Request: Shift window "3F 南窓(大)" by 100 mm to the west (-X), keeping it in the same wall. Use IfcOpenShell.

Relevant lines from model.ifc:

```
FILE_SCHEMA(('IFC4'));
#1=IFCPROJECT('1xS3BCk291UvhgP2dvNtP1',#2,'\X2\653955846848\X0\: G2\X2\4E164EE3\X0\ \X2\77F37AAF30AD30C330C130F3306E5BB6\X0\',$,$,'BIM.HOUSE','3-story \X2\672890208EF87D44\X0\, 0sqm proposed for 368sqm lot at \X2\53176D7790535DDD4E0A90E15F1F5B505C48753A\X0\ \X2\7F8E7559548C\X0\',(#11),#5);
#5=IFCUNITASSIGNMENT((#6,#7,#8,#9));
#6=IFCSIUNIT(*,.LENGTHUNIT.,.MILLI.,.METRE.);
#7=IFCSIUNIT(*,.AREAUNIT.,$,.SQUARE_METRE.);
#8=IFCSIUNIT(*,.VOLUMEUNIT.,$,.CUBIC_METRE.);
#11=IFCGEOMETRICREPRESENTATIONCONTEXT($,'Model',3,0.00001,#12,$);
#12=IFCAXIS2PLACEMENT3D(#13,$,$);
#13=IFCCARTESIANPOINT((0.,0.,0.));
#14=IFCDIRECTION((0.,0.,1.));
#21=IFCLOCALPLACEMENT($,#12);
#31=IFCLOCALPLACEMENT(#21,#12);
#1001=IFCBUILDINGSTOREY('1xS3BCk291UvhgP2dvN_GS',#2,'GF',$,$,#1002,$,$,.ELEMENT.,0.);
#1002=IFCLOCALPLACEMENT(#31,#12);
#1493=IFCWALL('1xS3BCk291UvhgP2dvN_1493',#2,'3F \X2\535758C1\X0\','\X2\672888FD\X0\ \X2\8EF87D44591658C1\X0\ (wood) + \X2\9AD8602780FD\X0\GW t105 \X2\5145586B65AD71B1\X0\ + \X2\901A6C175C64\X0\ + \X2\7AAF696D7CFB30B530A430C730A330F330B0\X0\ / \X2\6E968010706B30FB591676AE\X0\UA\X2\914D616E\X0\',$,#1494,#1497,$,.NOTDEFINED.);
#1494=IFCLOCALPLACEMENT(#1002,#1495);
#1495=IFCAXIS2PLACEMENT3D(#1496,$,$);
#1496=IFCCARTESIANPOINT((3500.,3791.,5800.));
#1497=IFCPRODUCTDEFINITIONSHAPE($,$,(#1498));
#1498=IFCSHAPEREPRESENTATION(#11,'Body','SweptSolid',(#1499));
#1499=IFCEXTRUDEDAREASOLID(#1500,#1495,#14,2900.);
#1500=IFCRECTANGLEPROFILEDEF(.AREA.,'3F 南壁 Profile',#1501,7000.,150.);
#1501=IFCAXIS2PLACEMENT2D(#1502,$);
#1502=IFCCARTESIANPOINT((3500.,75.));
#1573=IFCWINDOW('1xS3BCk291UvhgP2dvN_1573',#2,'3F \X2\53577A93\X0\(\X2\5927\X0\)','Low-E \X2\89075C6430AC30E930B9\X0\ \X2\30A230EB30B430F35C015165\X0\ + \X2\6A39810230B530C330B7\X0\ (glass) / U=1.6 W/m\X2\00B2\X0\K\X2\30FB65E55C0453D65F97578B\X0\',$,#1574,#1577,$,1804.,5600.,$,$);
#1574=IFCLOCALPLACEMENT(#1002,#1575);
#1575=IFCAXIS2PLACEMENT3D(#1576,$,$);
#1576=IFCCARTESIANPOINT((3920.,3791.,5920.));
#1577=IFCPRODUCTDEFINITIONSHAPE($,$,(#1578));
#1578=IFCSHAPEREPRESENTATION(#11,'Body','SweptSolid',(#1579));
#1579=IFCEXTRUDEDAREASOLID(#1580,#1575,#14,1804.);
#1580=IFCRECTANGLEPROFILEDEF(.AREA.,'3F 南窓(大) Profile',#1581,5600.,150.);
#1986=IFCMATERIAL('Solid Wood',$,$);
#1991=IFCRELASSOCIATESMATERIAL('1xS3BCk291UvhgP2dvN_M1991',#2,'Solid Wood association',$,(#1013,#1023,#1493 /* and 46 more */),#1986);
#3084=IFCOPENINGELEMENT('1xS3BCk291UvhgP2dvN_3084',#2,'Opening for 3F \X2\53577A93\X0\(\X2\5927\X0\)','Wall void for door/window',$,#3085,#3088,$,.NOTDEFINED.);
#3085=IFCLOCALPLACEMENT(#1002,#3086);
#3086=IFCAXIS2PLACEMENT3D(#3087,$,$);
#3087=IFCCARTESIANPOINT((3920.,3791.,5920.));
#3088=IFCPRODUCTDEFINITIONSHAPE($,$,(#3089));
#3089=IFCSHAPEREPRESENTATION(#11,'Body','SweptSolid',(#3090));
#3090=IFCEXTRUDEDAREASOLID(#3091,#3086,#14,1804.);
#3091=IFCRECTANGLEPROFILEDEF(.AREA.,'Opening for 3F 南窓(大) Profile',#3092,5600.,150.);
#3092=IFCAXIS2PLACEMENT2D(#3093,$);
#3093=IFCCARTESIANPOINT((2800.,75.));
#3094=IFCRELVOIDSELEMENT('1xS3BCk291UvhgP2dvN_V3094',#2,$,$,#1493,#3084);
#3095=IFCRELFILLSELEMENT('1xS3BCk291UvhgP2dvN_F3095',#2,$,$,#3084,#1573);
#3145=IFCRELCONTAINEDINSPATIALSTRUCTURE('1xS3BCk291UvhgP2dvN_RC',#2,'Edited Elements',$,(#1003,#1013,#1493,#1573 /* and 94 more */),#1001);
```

```python
import ifcopenshell
import ifcopenshell.api.geometry
import ifcopenshell.util.placement
import ifcopenshell.util.unit

model = ifcopenshell.open("model.ifc")
unit_scale = ifcopenshell.util.unit.calculate_unit_scale(model)

window = model.by_guid("1xS3BCk291UvhgP2dvN_1573")
opening = window.FillsVoids[0].RelatingOpeningElement
wall = opening.VoidsElements[0].RelatingBuildingElement

wall_matrix = ifcopenshell.util.placement.get_local_placement(wall.ObjectPlacement)
shift = wall_matrix[:3, 0] * -0.1 / unit_scale
before = ifcopenshell.util.placement.get_local_placement(window.ObjectPlacement)[:3, 3].copy()

# The window is not placed relative to its opening, so move both.
for product in (opening, window):
    matrix = ifcopenshell.util.placement.get_local_placement(product.ObjectPlacement)
    matrix[:3, 3] += shift
    ifcopenshell.api.geometry.edit_object_placement(model, product=product, matrix=matrix, is_si=False)

after = ifcopenshell.util.placement.get_local_placement(window.ObjectPlacement)[:3, 3]
print("window moved by", (after - before).round(3) + 0.0)

model.write("model_updated.ifc")
```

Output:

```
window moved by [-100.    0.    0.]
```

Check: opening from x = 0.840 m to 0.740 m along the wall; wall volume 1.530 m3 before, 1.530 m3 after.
